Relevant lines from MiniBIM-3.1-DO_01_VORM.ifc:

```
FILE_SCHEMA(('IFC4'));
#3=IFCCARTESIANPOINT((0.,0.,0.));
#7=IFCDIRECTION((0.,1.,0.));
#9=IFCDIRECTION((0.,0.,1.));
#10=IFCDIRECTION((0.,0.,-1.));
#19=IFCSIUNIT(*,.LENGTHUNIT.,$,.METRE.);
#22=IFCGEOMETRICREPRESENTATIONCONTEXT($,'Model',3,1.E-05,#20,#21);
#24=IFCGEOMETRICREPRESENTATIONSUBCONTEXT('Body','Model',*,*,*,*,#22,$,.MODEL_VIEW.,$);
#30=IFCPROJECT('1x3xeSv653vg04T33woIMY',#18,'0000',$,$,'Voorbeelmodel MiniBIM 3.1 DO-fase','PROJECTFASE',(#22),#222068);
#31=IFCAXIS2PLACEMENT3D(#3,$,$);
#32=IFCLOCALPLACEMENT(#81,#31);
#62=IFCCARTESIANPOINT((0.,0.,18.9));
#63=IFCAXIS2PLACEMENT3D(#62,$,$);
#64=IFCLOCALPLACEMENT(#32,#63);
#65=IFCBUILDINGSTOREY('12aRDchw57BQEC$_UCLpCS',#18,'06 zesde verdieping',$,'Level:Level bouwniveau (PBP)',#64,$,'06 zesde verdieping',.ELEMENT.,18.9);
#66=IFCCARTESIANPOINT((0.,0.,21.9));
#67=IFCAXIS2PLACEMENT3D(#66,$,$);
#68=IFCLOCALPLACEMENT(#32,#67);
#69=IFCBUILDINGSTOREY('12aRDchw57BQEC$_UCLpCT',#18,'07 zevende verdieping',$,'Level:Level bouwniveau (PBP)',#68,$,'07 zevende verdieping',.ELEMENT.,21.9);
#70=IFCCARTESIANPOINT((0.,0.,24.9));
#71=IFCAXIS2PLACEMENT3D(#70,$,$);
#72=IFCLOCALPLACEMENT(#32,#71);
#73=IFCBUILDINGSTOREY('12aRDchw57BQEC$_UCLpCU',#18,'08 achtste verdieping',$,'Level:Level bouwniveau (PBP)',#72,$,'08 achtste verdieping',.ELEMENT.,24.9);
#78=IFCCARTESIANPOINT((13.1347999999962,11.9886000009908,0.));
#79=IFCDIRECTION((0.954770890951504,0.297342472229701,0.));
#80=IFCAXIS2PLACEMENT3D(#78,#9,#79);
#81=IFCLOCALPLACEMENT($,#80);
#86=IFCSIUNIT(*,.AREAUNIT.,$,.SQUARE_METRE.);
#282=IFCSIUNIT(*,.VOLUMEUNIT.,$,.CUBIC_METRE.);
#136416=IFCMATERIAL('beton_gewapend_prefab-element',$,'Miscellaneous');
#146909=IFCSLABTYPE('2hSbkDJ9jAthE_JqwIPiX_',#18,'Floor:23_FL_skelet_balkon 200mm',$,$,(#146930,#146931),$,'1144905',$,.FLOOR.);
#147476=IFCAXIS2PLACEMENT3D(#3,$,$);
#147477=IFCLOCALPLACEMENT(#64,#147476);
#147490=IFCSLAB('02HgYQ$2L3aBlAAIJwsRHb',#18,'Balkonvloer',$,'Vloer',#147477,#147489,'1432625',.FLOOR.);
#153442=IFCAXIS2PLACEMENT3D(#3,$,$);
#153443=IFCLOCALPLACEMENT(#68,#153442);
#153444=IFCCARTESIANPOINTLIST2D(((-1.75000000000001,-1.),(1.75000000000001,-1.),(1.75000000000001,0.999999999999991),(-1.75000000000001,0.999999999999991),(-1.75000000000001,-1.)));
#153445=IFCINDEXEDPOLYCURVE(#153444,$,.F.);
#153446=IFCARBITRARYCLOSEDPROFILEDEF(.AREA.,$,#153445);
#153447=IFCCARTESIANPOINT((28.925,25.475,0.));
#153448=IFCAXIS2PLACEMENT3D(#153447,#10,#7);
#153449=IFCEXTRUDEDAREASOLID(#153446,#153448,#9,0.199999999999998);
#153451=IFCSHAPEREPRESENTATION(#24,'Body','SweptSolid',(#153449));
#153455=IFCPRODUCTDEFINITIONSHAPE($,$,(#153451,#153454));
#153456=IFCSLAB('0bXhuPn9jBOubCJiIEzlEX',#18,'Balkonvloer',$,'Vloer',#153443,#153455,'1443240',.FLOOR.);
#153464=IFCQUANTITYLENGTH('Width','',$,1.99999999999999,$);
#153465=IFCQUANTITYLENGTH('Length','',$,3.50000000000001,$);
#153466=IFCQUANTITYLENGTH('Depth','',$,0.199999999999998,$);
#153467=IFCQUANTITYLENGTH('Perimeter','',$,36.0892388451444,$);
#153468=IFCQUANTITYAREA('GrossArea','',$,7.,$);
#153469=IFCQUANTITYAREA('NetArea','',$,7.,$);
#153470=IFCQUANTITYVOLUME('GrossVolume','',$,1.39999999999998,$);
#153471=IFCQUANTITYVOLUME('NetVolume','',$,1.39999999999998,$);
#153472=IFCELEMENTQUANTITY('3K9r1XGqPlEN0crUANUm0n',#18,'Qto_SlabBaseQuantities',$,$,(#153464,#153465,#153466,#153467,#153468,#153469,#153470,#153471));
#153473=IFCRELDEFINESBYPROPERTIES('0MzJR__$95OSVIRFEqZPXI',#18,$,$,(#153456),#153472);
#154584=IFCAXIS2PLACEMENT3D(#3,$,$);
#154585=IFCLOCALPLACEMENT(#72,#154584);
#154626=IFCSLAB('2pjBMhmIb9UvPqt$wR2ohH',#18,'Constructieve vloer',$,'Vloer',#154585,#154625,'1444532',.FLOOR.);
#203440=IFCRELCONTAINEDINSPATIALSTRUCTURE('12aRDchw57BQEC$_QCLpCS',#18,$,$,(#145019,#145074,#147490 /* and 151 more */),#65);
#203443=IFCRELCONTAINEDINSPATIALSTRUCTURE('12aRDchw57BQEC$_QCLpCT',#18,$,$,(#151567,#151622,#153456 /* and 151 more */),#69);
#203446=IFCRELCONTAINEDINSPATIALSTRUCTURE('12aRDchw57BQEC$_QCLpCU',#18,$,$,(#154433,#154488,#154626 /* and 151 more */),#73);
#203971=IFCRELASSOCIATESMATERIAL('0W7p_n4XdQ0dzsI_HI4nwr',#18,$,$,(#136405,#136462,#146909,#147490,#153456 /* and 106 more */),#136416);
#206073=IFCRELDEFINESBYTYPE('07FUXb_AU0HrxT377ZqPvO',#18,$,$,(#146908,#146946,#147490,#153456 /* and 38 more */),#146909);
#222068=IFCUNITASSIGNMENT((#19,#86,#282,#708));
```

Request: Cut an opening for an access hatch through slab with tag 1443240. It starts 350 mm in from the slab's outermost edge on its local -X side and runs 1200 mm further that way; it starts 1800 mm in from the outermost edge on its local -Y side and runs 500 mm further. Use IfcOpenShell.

```python
import numpy as np
import ifcopenshell
import ifcopenshell.api.feature
import ifcopenshell.api.geometry
import ifcopenshell.api.pset
import ifcopenshell.api.root
import ifcopenshell.geom
import ifcopenshell.util.element
import ifcopenshell.util.placement
import ifcopenshell.util.representation
import ifcopenshell.util.shape
import ifcopenshell.util.unit

model = ifcopenshell.open("MiniBIM-3.1-DO_01_VORM.ifc")
unit_scale = ifcopenshell.util.unit.calculate_unit_scale(model)
area_scale = ifcopenshell.util.unit.calculate_unit_scale(model, "AREAUNIT")
volume_scale = ifcopenshell.util.unit.calculate_unit_scale(model, "VOLUMEUNIT")
settings = ifcopenshell.geom.settings()


def volume(element):
    """Net volume in cubic metres, openings subtracted."""
    shape = ifcopenshell.geom.create_shape(settings, element)
    return ifcopenshell.util.shape.get_volume(shape.geometry)


slab = model.by_guid("0bXhuPn9jBOubCJiIEzlEX")
before = volume(slab)

# Extent in the slab's own axes, in metres. The edges named are its -X and -Y sides.
slab_shape = ifcopenshell.geom.create_shape(settings, slab)
vertices = ifcopenshell.util.shape.get_vertices(slab_shape.geometry)
x_min, y_min, bottom = vertices.min(axis=0)
top = vertices[:, 2].max()

opening = ifcopenshell.api.root.create_entity(model, ifc_class="IfcOpeningElement", name="Access hatch opening", predefined_type="OPENING")
context = ifcopenshell.util.representation.get_context(model, "Model", "Body", "MODEL_VIEW")
width, depth = 1.2, 0.5
outline = [(0.0, 0.0), (width, 0.0), (width, depth), (0.0, depth), (0.0, 0.0)]
# Overshoot both faces by 50 mm so the cut is clean.
shape = ifcopenshell.api.geometry.add_slab_representation(
    model, context=context, depth=top - bottom + 0.1, polyline=outline
)
ifcopenshell.api.geometry.assign_representation(model, product=opening, representation=shape)

matrix = ifcopenshell.util.placement.get_local_placement(slab.ObjectPlacement)
matrix[:, 3] = matrix @ np.append(np.array([x_min + 0.35, y_min + 1.8, bottom - 0.05]) / unit_scale, 1.0)
ifcopenshell.api.geometry.edit_object_placement(model, product=opening, matrix=matrix, is_si=False)
ifcopenshell.api.feature.add_feature(model, feature=opening, element=slab)

after = volume(slab)

# Update the slab's stored quantities.
qto = model.by_id(ifcopenshell.util.element.get_pset(slab, "Qto_SlabBaseQuantities", should_inherit=False)["id"])
ifcopenshell.api.pset.edit_qto(model, qto=qto, properties={
    "NetArea": after / (top - bottom) / area_scale,
    "NetVolume": after / volume_scale,
})

print(f"slab volume {before:.3f} -> {after:.3f} m3")

model.write("MiniBIM-3.1-DO_01_VORM_edited.ifc")
```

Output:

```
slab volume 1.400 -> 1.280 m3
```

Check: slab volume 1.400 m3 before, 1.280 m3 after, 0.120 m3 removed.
